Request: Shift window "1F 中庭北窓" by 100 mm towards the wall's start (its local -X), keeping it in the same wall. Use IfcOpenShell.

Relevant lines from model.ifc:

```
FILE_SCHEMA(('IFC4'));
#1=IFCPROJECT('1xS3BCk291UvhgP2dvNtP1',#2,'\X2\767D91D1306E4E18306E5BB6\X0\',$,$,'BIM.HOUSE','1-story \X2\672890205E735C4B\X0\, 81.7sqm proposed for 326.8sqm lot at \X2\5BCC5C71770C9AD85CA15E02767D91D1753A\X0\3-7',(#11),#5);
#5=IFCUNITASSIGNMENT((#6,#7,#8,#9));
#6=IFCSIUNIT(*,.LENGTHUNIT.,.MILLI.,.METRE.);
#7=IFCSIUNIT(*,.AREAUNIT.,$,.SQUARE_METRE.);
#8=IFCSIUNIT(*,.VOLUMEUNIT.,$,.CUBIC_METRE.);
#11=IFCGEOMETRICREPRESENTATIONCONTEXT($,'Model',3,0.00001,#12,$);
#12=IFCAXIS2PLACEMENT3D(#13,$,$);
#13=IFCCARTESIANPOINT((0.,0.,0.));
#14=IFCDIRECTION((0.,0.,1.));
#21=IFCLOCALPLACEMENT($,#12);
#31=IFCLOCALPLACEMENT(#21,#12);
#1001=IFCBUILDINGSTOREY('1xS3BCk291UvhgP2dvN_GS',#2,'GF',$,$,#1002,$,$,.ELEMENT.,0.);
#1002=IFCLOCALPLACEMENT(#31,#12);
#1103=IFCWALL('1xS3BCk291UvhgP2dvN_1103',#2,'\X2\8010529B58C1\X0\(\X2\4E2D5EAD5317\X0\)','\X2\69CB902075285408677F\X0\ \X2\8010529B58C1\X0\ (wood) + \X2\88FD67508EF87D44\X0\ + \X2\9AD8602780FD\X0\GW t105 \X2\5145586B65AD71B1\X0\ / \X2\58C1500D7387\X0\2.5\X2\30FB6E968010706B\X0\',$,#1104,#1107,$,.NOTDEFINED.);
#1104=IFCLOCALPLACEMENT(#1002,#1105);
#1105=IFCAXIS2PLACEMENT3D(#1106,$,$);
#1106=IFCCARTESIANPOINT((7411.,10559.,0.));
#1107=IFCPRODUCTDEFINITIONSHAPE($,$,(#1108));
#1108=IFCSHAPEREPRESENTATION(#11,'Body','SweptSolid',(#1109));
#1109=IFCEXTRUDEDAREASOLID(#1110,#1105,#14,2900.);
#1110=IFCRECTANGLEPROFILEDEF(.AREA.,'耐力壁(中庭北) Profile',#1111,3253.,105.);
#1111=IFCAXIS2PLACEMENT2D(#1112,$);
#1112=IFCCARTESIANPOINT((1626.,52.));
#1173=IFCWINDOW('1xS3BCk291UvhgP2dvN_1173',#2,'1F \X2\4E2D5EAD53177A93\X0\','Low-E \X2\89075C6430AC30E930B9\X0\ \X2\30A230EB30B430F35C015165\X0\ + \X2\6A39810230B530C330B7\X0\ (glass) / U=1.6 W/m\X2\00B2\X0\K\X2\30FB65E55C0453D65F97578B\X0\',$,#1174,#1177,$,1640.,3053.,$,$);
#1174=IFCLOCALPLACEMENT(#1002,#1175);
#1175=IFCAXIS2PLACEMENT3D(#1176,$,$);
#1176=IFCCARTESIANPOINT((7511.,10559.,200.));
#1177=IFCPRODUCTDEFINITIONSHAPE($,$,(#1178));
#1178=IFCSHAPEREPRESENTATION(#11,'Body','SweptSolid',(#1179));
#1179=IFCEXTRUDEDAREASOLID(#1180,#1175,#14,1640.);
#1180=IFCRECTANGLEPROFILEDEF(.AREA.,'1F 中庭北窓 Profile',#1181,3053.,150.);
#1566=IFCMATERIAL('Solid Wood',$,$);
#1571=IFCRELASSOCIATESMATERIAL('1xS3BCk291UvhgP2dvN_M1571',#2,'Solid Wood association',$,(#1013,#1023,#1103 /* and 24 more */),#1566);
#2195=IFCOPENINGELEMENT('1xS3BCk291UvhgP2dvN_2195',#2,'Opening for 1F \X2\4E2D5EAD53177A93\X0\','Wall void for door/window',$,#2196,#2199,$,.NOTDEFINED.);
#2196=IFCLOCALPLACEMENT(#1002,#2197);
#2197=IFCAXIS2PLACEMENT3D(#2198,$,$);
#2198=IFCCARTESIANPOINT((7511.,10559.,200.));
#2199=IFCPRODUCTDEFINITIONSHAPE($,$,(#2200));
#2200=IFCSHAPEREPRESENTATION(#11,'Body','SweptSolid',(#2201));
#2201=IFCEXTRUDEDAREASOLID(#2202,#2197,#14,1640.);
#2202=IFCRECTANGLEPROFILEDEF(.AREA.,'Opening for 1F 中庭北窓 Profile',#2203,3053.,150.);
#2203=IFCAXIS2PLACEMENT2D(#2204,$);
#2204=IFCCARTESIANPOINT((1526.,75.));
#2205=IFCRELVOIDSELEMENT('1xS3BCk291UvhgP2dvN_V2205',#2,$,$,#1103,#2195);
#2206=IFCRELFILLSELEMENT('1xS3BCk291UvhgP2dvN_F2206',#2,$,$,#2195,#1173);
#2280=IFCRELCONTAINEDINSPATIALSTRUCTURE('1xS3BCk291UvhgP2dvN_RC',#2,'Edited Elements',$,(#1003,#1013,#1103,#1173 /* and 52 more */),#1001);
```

```python
import ifcopenshell
import ifcopenshell.api.geometry
import ifcopenshell.util.placement

model = ifcopenshell.open("model.ifc")

window = model.by_guid("1xS3BCk291UvhgP2dvN_1173")
opening = window.FillsVoids[0].RelatingOpeningElement
wall = opening.VoidsElements[0].RelatingBuildingElement

wall_matrix = ifcopenshell.util.placement.get_local_placement(wall.ObjectPlacement)
shift = wall_matrix[:3, 0] * -100.0
before = ifcopenshell.util.placement.get_local_placement(window.ObjectPlacement)[:3, 3].copy()

# The window is not placed relative to its opening, so move both.
for product in (opening, window):
    matrix = ifcopenshell.util.placement.get_local_placement(product.ObjectPlacement)
    matrix[:3, 3] += shift
    ifcopenshell.api.geometry.edit_object_placement(model, product=product, matrix=matrix, is_si=False)

after = ifcopenshell.util.placement.get_local_placement(window.ObjectPlacement)[:3, 3]
print("window moved by", (after - before).round(3) + 0.0)

model.write("model-out.ifc")
```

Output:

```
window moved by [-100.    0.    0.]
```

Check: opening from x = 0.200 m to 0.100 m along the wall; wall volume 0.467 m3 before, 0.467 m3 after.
